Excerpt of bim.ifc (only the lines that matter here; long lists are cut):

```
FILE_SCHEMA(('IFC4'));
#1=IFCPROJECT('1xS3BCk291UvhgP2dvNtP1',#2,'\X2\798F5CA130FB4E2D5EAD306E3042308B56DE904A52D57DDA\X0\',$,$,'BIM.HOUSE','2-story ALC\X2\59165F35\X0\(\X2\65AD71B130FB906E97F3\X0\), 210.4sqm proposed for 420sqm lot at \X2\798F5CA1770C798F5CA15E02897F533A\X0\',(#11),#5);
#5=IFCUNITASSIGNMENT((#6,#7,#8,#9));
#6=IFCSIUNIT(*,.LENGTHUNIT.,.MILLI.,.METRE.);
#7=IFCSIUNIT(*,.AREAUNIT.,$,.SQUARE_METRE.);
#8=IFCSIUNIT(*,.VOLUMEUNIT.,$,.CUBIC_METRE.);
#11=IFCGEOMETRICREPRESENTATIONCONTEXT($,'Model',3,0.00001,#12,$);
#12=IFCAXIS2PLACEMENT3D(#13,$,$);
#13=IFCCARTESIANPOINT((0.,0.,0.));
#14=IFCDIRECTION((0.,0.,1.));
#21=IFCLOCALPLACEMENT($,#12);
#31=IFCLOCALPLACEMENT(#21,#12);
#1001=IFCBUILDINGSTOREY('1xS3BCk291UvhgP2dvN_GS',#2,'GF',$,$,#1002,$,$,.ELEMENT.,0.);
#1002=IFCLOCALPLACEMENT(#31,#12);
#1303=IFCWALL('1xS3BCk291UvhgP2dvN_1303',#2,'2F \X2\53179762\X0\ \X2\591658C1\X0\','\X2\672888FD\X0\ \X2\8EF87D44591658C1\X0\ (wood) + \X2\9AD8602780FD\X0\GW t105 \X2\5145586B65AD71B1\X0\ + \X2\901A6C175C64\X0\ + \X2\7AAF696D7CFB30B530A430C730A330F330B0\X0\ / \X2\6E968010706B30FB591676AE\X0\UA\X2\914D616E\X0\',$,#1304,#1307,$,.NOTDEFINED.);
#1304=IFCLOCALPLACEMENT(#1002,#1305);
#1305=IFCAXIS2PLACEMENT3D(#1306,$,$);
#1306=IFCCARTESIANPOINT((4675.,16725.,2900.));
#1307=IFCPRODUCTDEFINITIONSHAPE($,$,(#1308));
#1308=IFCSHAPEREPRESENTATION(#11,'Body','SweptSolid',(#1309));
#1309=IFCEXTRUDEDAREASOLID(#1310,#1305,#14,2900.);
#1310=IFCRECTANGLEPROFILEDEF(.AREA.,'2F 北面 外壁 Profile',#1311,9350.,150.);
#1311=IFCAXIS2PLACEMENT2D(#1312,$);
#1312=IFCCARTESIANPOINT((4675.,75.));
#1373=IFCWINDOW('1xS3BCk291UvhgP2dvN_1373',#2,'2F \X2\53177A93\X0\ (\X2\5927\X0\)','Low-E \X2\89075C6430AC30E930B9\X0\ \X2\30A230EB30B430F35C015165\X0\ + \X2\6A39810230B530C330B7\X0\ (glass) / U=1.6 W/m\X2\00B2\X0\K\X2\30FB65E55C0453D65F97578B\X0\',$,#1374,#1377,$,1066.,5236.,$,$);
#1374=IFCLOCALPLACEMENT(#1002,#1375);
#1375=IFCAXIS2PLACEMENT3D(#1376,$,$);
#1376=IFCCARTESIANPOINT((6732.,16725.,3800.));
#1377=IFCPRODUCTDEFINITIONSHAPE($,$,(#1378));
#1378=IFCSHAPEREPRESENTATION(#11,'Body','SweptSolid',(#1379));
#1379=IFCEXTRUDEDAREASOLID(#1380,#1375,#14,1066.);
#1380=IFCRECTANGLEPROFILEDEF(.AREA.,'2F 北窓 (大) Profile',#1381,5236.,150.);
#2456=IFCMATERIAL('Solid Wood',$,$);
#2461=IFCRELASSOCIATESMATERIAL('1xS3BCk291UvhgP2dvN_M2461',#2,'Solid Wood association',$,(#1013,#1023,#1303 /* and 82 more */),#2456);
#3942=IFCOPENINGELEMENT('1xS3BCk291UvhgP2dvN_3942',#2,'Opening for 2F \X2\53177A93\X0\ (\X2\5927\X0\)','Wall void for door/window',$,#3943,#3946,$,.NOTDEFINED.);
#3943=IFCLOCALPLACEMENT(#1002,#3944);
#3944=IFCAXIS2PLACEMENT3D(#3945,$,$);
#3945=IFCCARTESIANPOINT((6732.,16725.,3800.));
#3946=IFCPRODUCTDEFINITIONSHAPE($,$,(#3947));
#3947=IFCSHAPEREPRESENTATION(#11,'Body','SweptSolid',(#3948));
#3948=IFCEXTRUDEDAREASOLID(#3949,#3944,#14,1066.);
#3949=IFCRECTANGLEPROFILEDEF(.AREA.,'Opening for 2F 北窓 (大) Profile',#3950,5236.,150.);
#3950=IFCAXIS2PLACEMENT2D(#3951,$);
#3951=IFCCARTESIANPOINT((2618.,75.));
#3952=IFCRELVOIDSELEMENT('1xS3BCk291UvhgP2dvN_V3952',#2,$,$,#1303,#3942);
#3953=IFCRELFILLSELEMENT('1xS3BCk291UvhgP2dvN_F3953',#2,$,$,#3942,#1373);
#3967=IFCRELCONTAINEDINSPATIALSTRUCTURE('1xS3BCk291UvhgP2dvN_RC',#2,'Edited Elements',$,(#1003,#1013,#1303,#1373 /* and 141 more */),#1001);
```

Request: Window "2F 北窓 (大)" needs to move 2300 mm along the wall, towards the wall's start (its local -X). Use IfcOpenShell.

```python
import ifcopenshell
import ifcopenshell.api.geometry
import ifcopenshell.util.placement

model = ifcopenshell.open("bim.ifc")

window = model.by_id(1373)
opening = window.FillsVoids[0].RelatingOpeningElement
wall = opening.VoidsElements[0].RelatingBuildingElement

wall_matrix = ifcopenshell.util.placement.get_local_placement(wall.ObjectPlacement)
shift = wall_matrix[:3, 0] * -2300.0
before = ifcopenshell.util.placement.get_local_placement(window.ObjectPlacement)[:3, 3].copy()

# The window is not placed relative to its opening, so move both.
for product in (opening, window):
    matrix = ifcopenshell.util.placement.get_local_placement(product.ObjectPlacement)
    matrix[:3, 3] += shift
    ifcopenshell.api.geometry.edit_object_placement(model, product=product, matrix=matrix, is_si=False)

after = ifcopenshell.util.placement.get_local_placement(window.ObjectPlacement)[:3, 3]
print("window moved by", (after - before).round(3) + 0.0)

model.write("bim-out.ifc")
```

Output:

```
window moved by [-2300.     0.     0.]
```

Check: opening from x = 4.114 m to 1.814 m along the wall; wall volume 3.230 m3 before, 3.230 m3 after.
